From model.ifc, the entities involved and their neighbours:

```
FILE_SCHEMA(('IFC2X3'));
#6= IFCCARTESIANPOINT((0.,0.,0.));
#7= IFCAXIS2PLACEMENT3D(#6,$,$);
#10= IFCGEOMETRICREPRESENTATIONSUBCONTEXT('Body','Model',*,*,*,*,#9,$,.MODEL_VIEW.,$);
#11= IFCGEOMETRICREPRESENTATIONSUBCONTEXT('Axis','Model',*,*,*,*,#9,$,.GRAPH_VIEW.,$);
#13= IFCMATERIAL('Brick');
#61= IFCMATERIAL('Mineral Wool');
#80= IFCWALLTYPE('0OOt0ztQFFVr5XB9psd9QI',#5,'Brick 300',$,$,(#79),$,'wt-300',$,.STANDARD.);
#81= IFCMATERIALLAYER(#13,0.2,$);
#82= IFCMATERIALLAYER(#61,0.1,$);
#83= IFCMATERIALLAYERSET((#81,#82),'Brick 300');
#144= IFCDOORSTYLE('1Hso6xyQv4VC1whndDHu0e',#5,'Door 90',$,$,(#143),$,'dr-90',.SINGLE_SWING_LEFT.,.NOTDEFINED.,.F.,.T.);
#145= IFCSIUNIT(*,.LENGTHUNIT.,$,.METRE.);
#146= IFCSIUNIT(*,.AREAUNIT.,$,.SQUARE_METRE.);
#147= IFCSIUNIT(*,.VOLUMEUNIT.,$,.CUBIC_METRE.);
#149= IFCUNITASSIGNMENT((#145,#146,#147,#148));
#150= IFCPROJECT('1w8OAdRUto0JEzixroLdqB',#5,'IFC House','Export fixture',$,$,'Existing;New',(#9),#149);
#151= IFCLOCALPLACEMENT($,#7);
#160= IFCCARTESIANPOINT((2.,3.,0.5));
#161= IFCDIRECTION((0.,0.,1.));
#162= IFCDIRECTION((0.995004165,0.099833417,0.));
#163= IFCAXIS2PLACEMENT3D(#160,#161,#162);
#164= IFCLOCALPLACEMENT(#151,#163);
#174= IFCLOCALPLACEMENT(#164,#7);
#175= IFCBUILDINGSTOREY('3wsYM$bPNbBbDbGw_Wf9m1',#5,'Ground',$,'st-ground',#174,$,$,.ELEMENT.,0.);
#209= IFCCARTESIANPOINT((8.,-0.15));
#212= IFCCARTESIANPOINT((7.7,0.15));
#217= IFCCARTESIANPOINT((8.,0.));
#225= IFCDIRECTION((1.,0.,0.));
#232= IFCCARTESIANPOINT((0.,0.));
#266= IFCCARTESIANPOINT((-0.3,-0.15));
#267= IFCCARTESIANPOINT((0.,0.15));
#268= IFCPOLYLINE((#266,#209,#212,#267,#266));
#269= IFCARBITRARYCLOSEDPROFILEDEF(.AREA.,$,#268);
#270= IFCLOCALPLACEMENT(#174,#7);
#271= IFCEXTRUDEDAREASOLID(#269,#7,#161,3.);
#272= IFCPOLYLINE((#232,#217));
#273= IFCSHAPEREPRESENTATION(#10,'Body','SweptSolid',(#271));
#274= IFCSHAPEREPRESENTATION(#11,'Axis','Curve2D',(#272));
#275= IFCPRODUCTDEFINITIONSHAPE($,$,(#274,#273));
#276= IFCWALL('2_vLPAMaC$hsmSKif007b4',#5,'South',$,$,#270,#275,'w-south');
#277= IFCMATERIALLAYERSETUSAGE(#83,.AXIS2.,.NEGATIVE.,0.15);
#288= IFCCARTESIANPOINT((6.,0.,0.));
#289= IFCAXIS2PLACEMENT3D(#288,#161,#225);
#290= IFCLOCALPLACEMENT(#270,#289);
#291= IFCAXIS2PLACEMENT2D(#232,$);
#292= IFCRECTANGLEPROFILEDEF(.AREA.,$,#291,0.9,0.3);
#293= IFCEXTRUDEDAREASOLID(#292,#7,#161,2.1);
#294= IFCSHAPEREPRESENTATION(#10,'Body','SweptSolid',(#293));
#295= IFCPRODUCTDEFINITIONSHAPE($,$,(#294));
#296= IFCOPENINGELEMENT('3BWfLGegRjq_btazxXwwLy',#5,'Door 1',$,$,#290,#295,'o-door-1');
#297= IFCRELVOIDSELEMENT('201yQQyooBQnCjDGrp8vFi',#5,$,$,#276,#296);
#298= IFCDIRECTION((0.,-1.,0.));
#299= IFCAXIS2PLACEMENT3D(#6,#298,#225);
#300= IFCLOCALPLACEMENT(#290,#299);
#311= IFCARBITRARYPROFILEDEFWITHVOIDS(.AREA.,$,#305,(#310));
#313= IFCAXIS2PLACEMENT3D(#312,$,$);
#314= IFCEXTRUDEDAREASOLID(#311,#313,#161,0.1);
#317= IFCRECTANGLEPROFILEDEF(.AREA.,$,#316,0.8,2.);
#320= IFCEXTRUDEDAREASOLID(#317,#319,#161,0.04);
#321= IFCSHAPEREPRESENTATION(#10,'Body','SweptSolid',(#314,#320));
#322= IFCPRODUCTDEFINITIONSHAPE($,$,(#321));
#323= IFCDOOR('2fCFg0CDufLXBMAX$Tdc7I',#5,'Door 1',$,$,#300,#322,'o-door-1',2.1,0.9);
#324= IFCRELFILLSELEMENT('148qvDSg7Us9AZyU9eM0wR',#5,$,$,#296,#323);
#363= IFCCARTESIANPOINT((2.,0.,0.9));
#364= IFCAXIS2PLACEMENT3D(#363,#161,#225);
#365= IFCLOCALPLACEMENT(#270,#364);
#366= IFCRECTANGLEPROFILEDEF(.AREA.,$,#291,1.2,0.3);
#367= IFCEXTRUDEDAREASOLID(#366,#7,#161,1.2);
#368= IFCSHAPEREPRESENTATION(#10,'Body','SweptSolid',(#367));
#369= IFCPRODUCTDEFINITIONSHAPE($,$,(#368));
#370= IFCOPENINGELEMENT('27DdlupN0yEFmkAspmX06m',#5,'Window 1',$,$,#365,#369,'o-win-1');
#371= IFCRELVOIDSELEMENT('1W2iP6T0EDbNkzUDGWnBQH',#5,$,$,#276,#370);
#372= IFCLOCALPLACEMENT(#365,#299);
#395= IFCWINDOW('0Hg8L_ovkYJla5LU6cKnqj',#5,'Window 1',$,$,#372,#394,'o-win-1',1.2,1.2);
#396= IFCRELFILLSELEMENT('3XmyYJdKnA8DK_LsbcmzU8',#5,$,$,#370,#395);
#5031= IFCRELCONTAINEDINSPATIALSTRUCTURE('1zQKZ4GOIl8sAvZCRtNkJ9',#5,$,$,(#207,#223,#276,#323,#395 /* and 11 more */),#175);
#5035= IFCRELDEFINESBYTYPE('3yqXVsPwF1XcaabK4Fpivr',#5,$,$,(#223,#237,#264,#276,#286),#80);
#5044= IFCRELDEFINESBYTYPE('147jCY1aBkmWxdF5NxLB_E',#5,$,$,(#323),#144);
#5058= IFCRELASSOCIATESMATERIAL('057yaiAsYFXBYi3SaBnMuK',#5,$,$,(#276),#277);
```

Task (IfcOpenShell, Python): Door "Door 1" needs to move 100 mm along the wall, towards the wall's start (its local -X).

```python
import ifcopenshell
import ifcopenshell.api.geometry
import ifcopenshell.util.placement
import ifcopenshell.util.unit

model = ifcopenshell.open("model.ifc")
unit_scale = ifcopenshell.util.unit.calculate_unit_scale(model)

door = model.by_id(323)
opening = door.FillsVoids[0].RelatingOpeningElement
wall = opening.VoidsElements[0].RelatingBuildingElement

wall_matrix = ifcopenshell.util.placement.get_local_placement(wall.ObjectPlacement)
shift = wall_matrix[:3, 0] * -0.1 / unit_scale
before = ifcopenshell.util.placement.get_local_placement(door.ObjectPlacement)[:3, 3].copy()

# The door is placed relative to its opening, so it follows when the opening moves.
matrix = ifcopenshell.util.placement.get_local_placement(opening.ObjectPlacement)
matrix[:3, 3] += shift
ifcopenshell.api.geometry.edit_object_placement(
    model, product=opening, matrix=matrix, is_si=False, should_transform_children=True
)

after = ifcopenshell.util.placement.get_local_placement(door.ObjectPlacement)[:3, 3]
print("door moved by", (after - before).round(3) + 0.0)

model.write("model_v2.ifc")
```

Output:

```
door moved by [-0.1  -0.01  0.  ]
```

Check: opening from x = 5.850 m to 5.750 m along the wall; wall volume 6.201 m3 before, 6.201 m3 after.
